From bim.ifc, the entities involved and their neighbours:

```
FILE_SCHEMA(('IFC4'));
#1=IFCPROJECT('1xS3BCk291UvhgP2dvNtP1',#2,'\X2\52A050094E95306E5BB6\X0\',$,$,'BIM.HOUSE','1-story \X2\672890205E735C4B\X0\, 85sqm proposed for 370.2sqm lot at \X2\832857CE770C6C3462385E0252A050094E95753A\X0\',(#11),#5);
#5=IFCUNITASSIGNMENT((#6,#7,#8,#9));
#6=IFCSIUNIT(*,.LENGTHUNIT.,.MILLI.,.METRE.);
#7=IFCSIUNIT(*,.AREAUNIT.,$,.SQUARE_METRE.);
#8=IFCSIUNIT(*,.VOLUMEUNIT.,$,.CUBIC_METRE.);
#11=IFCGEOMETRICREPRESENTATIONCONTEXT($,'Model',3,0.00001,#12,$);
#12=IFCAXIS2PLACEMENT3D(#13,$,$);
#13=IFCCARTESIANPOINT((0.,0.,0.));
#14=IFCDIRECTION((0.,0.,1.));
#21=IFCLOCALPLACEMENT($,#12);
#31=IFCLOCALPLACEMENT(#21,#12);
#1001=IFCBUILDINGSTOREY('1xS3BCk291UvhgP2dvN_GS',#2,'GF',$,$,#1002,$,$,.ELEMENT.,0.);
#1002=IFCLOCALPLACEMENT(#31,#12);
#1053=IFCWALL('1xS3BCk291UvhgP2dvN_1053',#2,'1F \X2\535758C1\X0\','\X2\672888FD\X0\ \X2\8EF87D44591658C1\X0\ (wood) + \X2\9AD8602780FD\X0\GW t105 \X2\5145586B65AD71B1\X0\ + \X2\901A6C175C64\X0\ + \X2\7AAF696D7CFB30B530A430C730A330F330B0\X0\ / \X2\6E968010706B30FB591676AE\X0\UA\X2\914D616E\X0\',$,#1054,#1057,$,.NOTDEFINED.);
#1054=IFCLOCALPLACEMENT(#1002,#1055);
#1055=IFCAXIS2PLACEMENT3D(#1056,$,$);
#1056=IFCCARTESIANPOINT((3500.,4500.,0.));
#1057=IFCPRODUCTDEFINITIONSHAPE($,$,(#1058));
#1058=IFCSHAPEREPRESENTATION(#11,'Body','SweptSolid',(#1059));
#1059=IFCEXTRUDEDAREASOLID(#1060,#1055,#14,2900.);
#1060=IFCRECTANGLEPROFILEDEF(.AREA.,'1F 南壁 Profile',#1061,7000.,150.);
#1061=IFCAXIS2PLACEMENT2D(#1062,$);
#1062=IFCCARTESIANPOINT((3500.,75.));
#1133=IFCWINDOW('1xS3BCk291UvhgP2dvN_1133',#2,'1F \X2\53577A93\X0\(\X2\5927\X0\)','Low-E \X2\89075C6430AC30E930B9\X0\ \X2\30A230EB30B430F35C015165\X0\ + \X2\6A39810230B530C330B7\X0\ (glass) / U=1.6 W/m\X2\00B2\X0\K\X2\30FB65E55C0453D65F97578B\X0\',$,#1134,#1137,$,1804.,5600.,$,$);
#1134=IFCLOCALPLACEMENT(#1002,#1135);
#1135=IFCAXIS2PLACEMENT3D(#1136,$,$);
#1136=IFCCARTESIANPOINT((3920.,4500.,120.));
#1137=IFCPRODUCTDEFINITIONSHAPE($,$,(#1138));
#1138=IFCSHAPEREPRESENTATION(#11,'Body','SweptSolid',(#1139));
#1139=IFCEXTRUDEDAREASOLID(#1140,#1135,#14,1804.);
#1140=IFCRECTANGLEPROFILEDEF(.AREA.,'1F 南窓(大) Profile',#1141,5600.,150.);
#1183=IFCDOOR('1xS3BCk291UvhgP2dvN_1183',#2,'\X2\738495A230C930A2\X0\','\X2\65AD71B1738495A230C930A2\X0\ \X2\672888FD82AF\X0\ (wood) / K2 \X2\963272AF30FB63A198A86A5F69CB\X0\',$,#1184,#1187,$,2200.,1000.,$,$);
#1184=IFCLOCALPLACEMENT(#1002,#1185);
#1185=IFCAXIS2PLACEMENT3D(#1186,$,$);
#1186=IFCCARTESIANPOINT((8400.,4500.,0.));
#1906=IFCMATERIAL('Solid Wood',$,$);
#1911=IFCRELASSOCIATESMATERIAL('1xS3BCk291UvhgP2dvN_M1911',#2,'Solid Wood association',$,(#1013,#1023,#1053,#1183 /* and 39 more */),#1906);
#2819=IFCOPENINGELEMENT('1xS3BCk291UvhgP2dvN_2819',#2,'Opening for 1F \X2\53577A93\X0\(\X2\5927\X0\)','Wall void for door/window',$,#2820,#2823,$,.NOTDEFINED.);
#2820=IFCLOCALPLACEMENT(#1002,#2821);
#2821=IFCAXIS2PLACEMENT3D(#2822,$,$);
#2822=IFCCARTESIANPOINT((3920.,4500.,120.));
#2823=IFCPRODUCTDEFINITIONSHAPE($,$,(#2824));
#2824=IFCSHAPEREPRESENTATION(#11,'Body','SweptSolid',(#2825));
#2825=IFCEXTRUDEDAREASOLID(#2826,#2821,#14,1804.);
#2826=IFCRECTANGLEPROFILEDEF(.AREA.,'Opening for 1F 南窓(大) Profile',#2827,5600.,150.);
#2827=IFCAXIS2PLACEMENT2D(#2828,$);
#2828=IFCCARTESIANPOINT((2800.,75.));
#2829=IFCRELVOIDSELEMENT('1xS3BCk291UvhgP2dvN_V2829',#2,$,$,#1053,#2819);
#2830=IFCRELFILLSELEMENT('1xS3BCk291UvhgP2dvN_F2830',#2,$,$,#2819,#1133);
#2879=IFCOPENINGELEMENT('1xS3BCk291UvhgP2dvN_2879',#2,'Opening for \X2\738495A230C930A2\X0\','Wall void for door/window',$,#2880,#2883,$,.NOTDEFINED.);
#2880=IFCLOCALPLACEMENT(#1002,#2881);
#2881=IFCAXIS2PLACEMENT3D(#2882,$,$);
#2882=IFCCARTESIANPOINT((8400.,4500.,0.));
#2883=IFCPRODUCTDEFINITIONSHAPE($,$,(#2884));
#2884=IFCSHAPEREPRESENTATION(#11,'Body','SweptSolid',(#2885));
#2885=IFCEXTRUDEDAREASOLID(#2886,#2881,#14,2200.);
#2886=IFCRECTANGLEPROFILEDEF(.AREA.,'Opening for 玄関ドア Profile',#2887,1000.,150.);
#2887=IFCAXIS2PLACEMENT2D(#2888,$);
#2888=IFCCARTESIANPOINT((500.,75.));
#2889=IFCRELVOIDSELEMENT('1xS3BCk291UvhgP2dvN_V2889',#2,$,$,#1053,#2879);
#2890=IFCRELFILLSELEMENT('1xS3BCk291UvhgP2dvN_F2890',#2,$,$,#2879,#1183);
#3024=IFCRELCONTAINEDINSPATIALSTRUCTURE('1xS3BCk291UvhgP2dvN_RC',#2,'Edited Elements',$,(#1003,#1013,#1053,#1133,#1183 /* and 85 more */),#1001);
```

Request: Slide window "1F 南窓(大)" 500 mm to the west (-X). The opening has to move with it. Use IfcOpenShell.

```python
import ifcopenshell
import ifcopenshell.api.geometry
import ifcopenshell.util.placement

model = ifcopenshell.open("bim.ifc")

window = model.by_id(1133)
opening = window.FillsVoids[0].RelatingOpeningElement
wall = opening.VoidsElements[0].RelatingBuildingElement

wall_matrix = ifcopenshell.util.placement.get_local_placement(wall.ObjectPlacement)
shift = wall_matrix[:3, 0] * -500.0
before = ifcopenshell.util.placement.get_local_placement(window.ObjectPlacement)[:3, 3].copy()

# The window is not placed relative to its opening, so move both.
for product in (opening, window):
    matrix = ifcopenshell.util.placement.get_local_placement(product.ObjectPlacement)
    matrix[:3, 3] += shift
    ifcopenshell.api.geometry.edit_object_placement(model, product=product, matrix=matrix, is_si=False)

after = ifcopenshell.util.placement.get_local_placement(window.ObjectPlacement)[:3, 3]
print("window moved by", (after - before).round(3) + 0.0)

model.write("bim-out.ifc")
```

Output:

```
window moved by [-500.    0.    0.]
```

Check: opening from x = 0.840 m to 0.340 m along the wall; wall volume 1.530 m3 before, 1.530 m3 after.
